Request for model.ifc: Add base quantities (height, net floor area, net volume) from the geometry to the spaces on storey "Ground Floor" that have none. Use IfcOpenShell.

First a look at what the model holds.

```python
import ifcopenshell
import ifcopenshell.util.element
import ifcopenshell.util.unit

model = ifcopenshell.open("model.ifc")
print(model.schema)
for unit_type in ("LENGTHUNIT", "AREAUNIT", "VOLUMEUNIT"):
    print(unit_type, ifcopenshell.util.unit.calculate_unit_scale(model, unit_type))
storey = next(s for s in model.by_type("IfcBuildingStorey") if s.Name == "Ground Floor")
spaces = [e for e in ifcopenshell.util.element.get_decomposition(storey) if e.is_a("IfcSpace")]
for e in sorted(spaces, key=lambda e: e.id()):
    print(e.id(), e.is_a(), e.Name, list(ifcopenshell.util.element.get_psets(e, qtos_only=True)), sep=" | ")
```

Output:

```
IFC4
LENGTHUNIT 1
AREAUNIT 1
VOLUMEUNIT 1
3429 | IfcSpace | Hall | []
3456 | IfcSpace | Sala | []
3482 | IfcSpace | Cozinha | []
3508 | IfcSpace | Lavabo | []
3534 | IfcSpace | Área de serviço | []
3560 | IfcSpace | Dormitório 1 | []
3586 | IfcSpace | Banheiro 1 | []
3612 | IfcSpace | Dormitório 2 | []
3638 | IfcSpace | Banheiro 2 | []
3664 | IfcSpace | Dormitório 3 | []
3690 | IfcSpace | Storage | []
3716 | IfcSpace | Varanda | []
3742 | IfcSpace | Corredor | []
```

```python
import ifcopenshell
import ifcopenshell.api.pset
import ifcopenshell.geom
import ifcopenshell.util.element
import ifcopenshell.util.shape
import ifcopenshell.util.unit

model = ifcopenshell.open("model.ifc")
unit_scale = ifcopenshell.util.unit.calculate_unit_scale(model)
area_scale = ifcopenshell.util.unit.calculate_unit_scale(model, "AREAUNIT")
volume_scale = ifcopenshell.util.unit.calculate_unit_scale(model, "VOLUMEUNIT")
settings = ifcopenshell.geom.settings()

storey = next(s for s in model.by_type("IfcBuildingStorey") if s.Name == "Ground Floor")
spaces = [e for e in ifcopenshell.util.element.get_decomposition(storey) if e.is_a("IfcSpace")]

for e in sorted(spaces, key=lambda e: e.id()):
    if ifcopenshell.util.element.get_psets(e, qtos_only=True, should_inherit=False):
        continue
    # Geometry comes back in metres, in the element's own axes.
    shape = ifcopenshell.geom.create_shape(settings, e)
    values = {
        "Height": ifcopenshell.util.shape.get_z(shape.geometry) / unit_scale,
        "NetFloorArea": ifcopenshell.util.shape.get_footprint_area(shape.geometry) / area_scale,
        "NetVolume": ifcopenshell.util.shape.get_volume(shape.geometry) / volume_scale,
    }
    qto = ifcopenshell.api.pset.add_qto(model, product=e, name="Qto_SpaceBaseQuantities")
    ifcopenshell.api.pset.edit_qto(model, qto=qto, properties=values)
    print(e.id(), {k: round(v, 3) for k, v in values.items()})

model.write("model_edited.ifc")
```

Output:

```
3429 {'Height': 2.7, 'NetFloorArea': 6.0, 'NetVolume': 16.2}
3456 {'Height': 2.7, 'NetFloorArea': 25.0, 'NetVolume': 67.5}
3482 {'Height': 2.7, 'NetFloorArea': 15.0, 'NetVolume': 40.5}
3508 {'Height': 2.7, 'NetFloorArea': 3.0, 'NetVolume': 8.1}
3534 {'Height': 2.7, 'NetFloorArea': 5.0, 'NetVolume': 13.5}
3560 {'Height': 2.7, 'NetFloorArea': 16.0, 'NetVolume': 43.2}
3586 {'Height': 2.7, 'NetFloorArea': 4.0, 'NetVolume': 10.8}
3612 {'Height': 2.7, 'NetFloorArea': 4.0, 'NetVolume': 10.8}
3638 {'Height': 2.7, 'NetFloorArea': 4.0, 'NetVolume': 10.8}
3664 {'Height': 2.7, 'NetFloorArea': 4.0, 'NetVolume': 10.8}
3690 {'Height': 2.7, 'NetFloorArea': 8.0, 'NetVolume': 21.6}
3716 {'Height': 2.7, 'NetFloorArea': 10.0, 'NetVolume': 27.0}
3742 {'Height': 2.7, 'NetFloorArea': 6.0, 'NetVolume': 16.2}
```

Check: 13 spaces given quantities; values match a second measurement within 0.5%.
